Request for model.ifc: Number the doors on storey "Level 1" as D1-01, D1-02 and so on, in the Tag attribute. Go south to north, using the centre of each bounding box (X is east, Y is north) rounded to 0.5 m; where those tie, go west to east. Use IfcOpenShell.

First a look at what the model holds.

```python
import ifcopenshell
import ifcopenshell.util.element
import ifcopenshell.util.placement

model = ifcopenshell.open("model.ifc")
print(model.schema)
storey = next(s for s in model.by_type("IfcBuildingStorey") if s.Name == "Level 1")
doors = [e for e in ifcopenshell.util.element.get_decomposition(storey) if e.is_a("IfcDoor")]
for e in sorted(doors, key=lambda e: e.id()):
    origin = ifcopenshell.util.placement.get_local_placement(e.ObjectPlacement)[:3, 3]
    print(e.id(), e.Tag, e.Name, origin.round(2) + 0.0, sep=" | ")
```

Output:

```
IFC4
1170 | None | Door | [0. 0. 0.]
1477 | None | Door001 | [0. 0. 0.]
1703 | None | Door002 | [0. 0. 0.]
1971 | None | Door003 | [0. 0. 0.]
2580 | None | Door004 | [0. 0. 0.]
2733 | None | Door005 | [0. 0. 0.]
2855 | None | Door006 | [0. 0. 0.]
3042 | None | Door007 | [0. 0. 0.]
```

```python
import ifcopenshell
import ifcopenshell.geom
import ifcopenshell.util.element
import ifcopenshell.util.shape

model = ifcopenshell.open("model.ifc")
settings = ifcopenshell.geom.settings()
settings.set("use-world-coords", True)


def centre(element):
    shape = ifcopenshell.geom.create_shape(settings, element)
    return ifcopenshell.util.shape.get_bbox_centroid(shape.geometry)


storey = next(s for s in model.by_type("IfcBuildingStorey") if s.Name == "Level 1")
doors = [e for e in ifcopenshell.util.element.get_decomposition(storey) if e.is_a("IfcDoor")]

# Insertion points can sit at a corner or the storey origin, so sort by the geometry (in metres).
centres = {e: centre(e) for e in doors}
doors.sort(key=lambda e: (round(centres[e][1] / 0.5), centres[e][0]))

for i, e in enumerate(doors, start=1):
    number = f"D1-{i:02d}"
    e.Tag = number
    print(e.id(), number)

model.write("model_rev.ifc")
```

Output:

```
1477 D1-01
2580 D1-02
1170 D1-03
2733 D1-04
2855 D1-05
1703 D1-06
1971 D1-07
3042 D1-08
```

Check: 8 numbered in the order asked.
